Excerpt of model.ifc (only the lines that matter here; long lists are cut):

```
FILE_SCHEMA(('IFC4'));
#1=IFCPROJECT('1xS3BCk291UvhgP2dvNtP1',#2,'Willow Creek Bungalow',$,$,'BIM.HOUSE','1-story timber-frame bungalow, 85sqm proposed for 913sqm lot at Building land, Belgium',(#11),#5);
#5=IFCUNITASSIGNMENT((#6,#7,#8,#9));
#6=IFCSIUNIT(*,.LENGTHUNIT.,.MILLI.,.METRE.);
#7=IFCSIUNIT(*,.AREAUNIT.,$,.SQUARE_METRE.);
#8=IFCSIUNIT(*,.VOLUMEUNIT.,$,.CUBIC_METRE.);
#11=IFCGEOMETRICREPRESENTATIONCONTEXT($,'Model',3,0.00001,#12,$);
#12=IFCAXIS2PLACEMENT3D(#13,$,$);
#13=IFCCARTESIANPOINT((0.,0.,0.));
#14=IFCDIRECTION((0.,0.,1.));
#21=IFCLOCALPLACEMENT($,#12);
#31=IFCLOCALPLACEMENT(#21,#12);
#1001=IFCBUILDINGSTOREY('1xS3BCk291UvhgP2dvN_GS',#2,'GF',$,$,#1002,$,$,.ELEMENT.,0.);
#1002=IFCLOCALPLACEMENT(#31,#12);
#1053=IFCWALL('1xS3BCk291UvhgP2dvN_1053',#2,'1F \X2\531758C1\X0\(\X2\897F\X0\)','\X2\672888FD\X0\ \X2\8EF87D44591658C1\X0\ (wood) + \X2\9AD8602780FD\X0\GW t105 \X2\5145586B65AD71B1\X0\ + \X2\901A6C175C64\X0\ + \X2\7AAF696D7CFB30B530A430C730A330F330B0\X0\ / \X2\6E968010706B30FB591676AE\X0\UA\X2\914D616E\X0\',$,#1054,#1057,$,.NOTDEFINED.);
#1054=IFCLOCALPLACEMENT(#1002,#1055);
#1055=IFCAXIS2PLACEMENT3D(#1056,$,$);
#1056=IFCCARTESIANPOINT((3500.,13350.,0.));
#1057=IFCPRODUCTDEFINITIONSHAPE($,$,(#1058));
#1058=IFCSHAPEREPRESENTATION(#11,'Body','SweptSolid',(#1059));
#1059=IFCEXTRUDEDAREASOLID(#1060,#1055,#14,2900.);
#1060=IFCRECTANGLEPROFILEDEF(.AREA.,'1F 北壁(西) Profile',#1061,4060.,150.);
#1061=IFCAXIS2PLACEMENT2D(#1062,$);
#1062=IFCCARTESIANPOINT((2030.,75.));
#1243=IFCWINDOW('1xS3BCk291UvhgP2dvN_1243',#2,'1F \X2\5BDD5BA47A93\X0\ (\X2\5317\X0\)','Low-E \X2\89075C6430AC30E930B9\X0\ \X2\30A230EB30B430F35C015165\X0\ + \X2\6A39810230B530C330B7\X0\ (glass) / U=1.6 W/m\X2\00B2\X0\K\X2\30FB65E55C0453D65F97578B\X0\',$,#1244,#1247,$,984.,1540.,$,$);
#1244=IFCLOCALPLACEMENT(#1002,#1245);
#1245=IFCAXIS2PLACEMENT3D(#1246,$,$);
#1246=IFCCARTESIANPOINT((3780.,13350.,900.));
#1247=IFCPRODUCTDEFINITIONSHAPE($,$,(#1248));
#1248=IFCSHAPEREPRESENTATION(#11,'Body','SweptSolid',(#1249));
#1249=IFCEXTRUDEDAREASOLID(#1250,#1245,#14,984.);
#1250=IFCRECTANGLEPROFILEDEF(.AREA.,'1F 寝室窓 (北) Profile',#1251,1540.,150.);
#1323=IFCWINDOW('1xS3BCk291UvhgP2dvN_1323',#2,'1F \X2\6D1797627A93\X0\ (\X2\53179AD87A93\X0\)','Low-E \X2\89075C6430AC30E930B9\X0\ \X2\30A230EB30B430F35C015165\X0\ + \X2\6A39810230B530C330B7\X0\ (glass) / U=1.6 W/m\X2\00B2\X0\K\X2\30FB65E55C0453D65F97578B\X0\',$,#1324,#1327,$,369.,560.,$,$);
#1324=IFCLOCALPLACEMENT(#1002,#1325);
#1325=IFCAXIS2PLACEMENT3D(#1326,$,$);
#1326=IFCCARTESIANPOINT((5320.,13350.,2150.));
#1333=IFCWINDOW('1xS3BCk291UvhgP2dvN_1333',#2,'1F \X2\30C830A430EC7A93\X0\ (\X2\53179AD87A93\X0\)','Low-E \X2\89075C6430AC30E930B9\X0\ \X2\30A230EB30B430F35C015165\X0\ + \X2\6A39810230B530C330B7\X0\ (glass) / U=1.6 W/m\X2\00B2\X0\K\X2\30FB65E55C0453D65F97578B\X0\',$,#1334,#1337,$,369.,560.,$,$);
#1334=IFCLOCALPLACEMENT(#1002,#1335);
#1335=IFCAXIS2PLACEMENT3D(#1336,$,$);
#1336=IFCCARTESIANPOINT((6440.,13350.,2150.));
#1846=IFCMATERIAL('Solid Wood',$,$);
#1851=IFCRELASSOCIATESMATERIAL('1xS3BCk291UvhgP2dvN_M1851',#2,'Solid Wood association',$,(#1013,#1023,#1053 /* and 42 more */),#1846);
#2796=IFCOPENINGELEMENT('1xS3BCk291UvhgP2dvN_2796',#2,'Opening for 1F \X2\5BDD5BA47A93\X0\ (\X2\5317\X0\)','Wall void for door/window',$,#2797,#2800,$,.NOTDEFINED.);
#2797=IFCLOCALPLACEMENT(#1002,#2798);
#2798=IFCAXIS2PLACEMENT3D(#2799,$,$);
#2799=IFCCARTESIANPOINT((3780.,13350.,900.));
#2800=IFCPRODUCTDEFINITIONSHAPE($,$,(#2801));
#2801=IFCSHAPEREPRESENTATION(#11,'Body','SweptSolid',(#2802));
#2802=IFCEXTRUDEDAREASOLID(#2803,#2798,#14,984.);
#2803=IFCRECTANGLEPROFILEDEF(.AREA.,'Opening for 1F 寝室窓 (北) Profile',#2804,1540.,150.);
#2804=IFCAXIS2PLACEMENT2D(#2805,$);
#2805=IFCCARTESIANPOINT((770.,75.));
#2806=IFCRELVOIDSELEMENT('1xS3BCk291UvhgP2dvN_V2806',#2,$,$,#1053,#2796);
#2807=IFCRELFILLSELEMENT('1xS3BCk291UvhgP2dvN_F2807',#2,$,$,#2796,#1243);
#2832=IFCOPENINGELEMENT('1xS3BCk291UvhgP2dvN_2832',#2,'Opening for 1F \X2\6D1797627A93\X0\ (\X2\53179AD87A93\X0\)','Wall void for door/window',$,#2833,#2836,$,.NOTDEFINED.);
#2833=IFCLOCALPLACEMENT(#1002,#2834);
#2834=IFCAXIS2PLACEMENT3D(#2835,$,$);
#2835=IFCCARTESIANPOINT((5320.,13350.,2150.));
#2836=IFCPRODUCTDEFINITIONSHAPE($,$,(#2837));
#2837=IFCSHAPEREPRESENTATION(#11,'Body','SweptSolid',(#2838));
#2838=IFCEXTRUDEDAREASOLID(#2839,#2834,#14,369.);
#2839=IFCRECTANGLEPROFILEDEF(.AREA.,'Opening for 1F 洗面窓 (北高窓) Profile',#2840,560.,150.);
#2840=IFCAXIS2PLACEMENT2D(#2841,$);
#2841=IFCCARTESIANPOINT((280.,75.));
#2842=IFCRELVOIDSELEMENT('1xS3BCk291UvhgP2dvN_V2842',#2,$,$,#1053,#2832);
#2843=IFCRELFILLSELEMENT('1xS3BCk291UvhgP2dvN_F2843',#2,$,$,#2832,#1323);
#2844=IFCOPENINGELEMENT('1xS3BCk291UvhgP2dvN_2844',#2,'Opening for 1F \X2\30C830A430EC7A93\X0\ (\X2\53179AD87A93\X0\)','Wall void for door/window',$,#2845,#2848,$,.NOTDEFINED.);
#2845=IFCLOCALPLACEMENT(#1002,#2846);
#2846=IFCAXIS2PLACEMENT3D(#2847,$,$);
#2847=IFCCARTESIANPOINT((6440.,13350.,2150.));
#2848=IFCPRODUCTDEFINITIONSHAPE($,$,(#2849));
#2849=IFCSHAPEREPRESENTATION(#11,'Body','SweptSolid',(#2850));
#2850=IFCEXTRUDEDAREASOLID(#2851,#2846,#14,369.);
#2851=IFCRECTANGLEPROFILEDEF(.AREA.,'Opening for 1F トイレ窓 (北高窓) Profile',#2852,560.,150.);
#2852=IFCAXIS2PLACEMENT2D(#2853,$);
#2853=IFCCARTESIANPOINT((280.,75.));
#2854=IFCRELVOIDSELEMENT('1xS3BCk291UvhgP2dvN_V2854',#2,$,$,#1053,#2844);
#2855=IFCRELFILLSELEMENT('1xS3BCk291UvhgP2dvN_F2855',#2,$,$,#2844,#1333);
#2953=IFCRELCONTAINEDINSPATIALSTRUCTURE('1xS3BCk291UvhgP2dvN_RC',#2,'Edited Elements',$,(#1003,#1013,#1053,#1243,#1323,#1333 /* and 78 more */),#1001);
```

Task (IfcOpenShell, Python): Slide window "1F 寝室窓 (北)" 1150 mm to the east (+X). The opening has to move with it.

```python
import ifcopenshell
import ifcopenshell.api.geometry
import ifcopenshell.util.placement

model = ifcopenshell.open("model.ifc")

window = model.by_guid("1xS3BCk291UvhgP2dvN_1243")
opening = window.FillsVoids[0].RelatingOpeningElement
wall = opening.VoidsElements[0].RelatingBuildingElement

wall_matrix = ifcopenshell.util.placement.get_local_placement(wall.ObjectPlacement)
shift = wall_matrix[:3, 0] * 1150.0
before = ifcopenshell.util.placement.get_local_placement(window.ObjectPlacement)[:3, 3].copy()

# The window is not placed relative to its opening, so move both.
for product in (opening, window):
    matrix = ifcopenshell.util.placement.get_local_placement(product.ObjectPlacement)
    matrix[:3, 3] += shift
    ifcopenshell.api.geometry.edit_object_placement(model, product=product, matrix=matrix, is_si=False)

after = ifcopenshell.util.placement.get_local_placement(window.ObjectPlacement)[:3, 3]
print("window moved by", (after - before).round(3) + 0.0)

model.write("model_rev.ifc")
```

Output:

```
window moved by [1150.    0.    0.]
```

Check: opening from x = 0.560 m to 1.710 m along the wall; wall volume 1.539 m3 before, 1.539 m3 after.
